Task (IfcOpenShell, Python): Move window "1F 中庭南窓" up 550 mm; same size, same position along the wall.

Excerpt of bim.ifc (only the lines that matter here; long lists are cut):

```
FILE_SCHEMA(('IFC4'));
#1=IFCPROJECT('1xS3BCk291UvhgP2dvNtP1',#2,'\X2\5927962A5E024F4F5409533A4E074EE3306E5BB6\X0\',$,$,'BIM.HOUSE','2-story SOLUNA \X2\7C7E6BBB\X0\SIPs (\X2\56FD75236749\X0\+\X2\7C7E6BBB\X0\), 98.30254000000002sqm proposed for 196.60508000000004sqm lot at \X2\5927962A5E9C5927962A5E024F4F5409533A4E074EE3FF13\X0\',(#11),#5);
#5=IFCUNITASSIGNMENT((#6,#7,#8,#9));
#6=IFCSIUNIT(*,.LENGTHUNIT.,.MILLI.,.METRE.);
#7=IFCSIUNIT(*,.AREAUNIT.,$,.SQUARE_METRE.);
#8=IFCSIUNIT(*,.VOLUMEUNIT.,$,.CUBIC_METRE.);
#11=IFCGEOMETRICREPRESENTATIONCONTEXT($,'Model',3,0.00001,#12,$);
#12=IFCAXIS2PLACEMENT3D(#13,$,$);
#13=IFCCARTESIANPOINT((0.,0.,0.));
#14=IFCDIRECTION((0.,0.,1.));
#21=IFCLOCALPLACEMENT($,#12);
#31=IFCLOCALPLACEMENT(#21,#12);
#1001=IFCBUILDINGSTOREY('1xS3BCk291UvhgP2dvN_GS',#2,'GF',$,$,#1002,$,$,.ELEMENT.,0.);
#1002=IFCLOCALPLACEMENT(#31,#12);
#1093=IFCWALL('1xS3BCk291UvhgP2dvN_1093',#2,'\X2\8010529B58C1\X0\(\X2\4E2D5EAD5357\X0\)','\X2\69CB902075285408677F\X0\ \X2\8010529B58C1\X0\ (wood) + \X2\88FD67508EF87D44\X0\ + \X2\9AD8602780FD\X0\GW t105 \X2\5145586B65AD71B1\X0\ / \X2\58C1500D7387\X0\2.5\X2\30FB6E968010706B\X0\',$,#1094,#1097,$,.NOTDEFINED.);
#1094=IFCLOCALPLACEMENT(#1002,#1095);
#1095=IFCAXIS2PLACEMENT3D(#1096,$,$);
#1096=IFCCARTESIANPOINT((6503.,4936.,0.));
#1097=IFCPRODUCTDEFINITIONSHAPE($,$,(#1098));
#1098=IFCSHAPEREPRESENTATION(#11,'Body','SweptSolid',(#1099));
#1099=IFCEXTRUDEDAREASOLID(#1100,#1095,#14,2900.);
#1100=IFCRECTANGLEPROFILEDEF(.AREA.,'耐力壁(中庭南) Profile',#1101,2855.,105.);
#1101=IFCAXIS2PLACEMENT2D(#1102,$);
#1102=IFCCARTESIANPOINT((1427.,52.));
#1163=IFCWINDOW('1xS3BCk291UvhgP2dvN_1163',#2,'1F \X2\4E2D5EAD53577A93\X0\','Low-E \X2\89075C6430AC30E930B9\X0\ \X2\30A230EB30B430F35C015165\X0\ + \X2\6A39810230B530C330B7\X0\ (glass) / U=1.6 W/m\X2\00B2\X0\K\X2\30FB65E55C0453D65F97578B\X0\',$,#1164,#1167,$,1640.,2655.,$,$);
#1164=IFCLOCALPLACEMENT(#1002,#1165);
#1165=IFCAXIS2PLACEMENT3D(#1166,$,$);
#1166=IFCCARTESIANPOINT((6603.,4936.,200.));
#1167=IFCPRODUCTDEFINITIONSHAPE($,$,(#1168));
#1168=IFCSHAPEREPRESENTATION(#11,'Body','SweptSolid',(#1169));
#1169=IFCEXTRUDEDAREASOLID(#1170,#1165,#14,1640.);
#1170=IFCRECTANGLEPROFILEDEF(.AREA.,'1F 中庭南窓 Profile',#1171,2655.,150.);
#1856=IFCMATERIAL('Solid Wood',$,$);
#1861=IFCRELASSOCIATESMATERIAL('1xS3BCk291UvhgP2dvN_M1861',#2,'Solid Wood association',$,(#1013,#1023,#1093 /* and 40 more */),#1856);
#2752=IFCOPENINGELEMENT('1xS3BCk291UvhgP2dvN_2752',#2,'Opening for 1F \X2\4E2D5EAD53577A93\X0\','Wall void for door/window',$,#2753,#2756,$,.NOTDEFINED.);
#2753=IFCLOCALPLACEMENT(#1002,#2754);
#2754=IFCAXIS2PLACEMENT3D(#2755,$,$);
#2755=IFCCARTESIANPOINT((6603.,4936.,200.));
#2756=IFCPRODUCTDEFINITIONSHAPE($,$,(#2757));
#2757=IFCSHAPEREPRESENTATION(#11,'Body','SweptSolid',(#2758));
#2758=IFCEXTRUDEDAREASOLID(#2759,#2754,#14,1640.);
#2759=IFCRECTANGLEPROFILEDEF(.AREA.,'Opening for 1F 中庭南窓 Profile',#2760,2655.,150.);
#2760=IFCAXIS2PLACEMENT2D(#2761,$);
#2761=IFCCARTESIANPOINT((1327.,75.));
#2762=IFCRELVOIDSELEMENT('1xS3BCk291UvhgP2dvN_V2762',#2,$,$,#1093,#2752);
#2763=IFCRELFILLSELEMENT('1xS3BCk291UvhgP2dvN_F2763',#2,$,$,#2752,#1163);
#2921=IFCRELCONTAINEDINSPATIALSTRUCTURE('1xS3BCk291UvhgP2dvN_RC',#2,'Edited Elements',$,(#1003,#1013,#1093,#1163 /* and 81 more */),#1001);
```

```python
import numpy as np
import ifcopenshell
import ifcopenshell.api.geometry
import ifcopenshell.util.placement
import ifcopenshell.util.unit

model = ifcopenshell.open("bim.ifc")
unit_scale = ifcopenshell.util.unit.calculate_unit_scale(model)

window = model.by_id(1163)
opening = window.FillsVoids[0].RelatingOpeningElement
dz = 550.0

shift = np.array([0.0, 0.0, dz])
# The window is not placed relative to its opening, so move both.
for product in (opening, window):
    matrix = ifcopenshell.util.placement.get_local_placement(product.ObjectPlacement)
    matrix[:3, 3] += shift
    ifcopenshell.api.geometry.edit_object_placement(model, product=product, matrix=matrix, is_si=False)

print(f"moved by {dz * unit_scale:+.3f} m")

model.write("bim_edited.ifc")
```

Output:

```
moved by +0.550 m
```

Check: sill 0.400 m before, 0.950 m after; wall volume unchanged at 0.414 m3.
